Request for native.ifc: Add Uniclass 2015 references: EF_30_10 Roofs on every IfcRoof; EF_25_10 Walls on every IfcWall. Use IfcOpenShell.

First a look at what the model holds.

```python
import ifcopenshell

model = ifcopenshell.open("native.ifc")
print(model.schema)
print("classifications:", [c.Name for c in model.by_type("IfcClassification")])
for ifc_class in ("IfcDoor", "IfcRoof", "IfcStair", "IfcWall", "IfcWindow"):
    print(ifc_class, len(model.by_type(ifc_class)))
```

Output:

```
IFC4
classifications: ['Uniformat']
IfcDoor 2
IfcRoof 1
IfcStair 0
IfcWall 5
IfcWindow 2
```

```python
import ifcopenshell
import ifcopenshell.api.classification

model = ifcopenshell.open("native.ifc")

system = ifcopenshell.api.classification.add_classification(model, classification="Uniclass 2015")

codes = {
    "IfcRoof": ("EF_30_10", "Roofs"),
    "IfcWall": ("EF_25_10", "Walls"),
}
for ifc_class, (code, name) in codes.items():
    products = model.by_type(ifc_class)
    ifcopenshell.api.classification.add_reference(
        model, products=products, classification=system, identification=code, name=name
    )
    print(code, len(products))

model.write("native_v2.ifc")
```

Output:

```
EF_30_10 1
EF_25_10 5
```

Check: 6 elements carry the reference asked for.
